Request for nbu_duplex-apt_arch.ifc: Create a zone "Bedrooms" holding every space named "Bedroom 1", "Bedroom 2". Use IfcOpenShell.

First a look at what the model holds.

```python
import ifcopenshell

model = ifcopenshell.open("nbu_duplex-apt_arch.ifc")
print(model.schema)
seen = {}
for space in model.by_type("IfcSpace"):
    seen[space.LongName] = seen.get(space.LongName, 0) + 1
for name, count in sorted(seen.items(), key=str):
    print(count, "x", name)
print("zones:", [z.Name for z in model.by_type("IfcZone")][:20])
```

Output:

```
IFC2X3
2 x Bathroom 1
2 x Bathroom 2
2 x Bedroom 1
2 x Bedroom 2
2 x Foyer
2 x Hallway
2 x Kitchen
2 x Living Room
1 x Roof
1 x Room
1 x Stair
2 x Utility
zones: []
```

```python
import ifcopenshell
import ifcopenshell.api.group
import ifcopenshell.api.root

model = ifcopenshell.open("nbu_duplex-apt_arch.ifc")

names = {"Bedroom 1", "Bedroom 2"}
spaces = [s for s in model.by_type("IfcSpace") if s.LongName in names]

zone = ifcopenshell.api.root.create_entity(model, ifc_class="IfcZone", name="Bedrooms")
ifcopenshell.api.group.assign_group(model, products=spaces, group=zone)
print(len(spaces), "spaces in", zone.Name)

model.write("nbu_duplex-apt_arch_edited.ifc")
```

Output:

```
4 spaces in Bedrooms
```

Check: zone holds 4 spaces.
